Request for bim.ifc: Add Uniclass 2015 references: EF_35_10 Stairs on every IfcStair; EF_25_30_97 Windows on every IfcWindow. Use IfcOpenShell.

First a look at what the model holds.

```python
import ifcopenshell

model = ifcopenshell.open("bim.ifc")
print(model.schema)
print("classifications:", [c.Name for c in model.by_type("IfcClassification")])
for ifc_class in ("IfcDoor", "IfcRoof", "IfcStair", "IfcWall", "IfcWindow"):
    print(ifc_class, len(model.by_type(ifc_class)))
```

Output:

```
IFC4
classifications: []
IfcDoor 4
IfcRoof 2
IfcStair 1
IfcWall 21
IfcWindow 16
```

```python
import ifcopenshell
import ifcopenshell.api.classification

model = ifcopenshell.open("bim.ifc")

system = ifcopenshell.api.classification.add_classification(model, classification="Uniclass 2015")

codes = {
    "IfcStair": ("EF_35_10", "Stairs"),
    "IfcWindow": ("EF_25_30_97", "Windows"),
}
for ifc_class, (code, name) in codes.items():
    products = model.by_type(ifc_class)
    ifcopenshell.api.classification.add_reference(
        model, products=products, classification=system, identification=code, name=name
    )
    print(code, len(products))

model.write("bim-out.ifc")
```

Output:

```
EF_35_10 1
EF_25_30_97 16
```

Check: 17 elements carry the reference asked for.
